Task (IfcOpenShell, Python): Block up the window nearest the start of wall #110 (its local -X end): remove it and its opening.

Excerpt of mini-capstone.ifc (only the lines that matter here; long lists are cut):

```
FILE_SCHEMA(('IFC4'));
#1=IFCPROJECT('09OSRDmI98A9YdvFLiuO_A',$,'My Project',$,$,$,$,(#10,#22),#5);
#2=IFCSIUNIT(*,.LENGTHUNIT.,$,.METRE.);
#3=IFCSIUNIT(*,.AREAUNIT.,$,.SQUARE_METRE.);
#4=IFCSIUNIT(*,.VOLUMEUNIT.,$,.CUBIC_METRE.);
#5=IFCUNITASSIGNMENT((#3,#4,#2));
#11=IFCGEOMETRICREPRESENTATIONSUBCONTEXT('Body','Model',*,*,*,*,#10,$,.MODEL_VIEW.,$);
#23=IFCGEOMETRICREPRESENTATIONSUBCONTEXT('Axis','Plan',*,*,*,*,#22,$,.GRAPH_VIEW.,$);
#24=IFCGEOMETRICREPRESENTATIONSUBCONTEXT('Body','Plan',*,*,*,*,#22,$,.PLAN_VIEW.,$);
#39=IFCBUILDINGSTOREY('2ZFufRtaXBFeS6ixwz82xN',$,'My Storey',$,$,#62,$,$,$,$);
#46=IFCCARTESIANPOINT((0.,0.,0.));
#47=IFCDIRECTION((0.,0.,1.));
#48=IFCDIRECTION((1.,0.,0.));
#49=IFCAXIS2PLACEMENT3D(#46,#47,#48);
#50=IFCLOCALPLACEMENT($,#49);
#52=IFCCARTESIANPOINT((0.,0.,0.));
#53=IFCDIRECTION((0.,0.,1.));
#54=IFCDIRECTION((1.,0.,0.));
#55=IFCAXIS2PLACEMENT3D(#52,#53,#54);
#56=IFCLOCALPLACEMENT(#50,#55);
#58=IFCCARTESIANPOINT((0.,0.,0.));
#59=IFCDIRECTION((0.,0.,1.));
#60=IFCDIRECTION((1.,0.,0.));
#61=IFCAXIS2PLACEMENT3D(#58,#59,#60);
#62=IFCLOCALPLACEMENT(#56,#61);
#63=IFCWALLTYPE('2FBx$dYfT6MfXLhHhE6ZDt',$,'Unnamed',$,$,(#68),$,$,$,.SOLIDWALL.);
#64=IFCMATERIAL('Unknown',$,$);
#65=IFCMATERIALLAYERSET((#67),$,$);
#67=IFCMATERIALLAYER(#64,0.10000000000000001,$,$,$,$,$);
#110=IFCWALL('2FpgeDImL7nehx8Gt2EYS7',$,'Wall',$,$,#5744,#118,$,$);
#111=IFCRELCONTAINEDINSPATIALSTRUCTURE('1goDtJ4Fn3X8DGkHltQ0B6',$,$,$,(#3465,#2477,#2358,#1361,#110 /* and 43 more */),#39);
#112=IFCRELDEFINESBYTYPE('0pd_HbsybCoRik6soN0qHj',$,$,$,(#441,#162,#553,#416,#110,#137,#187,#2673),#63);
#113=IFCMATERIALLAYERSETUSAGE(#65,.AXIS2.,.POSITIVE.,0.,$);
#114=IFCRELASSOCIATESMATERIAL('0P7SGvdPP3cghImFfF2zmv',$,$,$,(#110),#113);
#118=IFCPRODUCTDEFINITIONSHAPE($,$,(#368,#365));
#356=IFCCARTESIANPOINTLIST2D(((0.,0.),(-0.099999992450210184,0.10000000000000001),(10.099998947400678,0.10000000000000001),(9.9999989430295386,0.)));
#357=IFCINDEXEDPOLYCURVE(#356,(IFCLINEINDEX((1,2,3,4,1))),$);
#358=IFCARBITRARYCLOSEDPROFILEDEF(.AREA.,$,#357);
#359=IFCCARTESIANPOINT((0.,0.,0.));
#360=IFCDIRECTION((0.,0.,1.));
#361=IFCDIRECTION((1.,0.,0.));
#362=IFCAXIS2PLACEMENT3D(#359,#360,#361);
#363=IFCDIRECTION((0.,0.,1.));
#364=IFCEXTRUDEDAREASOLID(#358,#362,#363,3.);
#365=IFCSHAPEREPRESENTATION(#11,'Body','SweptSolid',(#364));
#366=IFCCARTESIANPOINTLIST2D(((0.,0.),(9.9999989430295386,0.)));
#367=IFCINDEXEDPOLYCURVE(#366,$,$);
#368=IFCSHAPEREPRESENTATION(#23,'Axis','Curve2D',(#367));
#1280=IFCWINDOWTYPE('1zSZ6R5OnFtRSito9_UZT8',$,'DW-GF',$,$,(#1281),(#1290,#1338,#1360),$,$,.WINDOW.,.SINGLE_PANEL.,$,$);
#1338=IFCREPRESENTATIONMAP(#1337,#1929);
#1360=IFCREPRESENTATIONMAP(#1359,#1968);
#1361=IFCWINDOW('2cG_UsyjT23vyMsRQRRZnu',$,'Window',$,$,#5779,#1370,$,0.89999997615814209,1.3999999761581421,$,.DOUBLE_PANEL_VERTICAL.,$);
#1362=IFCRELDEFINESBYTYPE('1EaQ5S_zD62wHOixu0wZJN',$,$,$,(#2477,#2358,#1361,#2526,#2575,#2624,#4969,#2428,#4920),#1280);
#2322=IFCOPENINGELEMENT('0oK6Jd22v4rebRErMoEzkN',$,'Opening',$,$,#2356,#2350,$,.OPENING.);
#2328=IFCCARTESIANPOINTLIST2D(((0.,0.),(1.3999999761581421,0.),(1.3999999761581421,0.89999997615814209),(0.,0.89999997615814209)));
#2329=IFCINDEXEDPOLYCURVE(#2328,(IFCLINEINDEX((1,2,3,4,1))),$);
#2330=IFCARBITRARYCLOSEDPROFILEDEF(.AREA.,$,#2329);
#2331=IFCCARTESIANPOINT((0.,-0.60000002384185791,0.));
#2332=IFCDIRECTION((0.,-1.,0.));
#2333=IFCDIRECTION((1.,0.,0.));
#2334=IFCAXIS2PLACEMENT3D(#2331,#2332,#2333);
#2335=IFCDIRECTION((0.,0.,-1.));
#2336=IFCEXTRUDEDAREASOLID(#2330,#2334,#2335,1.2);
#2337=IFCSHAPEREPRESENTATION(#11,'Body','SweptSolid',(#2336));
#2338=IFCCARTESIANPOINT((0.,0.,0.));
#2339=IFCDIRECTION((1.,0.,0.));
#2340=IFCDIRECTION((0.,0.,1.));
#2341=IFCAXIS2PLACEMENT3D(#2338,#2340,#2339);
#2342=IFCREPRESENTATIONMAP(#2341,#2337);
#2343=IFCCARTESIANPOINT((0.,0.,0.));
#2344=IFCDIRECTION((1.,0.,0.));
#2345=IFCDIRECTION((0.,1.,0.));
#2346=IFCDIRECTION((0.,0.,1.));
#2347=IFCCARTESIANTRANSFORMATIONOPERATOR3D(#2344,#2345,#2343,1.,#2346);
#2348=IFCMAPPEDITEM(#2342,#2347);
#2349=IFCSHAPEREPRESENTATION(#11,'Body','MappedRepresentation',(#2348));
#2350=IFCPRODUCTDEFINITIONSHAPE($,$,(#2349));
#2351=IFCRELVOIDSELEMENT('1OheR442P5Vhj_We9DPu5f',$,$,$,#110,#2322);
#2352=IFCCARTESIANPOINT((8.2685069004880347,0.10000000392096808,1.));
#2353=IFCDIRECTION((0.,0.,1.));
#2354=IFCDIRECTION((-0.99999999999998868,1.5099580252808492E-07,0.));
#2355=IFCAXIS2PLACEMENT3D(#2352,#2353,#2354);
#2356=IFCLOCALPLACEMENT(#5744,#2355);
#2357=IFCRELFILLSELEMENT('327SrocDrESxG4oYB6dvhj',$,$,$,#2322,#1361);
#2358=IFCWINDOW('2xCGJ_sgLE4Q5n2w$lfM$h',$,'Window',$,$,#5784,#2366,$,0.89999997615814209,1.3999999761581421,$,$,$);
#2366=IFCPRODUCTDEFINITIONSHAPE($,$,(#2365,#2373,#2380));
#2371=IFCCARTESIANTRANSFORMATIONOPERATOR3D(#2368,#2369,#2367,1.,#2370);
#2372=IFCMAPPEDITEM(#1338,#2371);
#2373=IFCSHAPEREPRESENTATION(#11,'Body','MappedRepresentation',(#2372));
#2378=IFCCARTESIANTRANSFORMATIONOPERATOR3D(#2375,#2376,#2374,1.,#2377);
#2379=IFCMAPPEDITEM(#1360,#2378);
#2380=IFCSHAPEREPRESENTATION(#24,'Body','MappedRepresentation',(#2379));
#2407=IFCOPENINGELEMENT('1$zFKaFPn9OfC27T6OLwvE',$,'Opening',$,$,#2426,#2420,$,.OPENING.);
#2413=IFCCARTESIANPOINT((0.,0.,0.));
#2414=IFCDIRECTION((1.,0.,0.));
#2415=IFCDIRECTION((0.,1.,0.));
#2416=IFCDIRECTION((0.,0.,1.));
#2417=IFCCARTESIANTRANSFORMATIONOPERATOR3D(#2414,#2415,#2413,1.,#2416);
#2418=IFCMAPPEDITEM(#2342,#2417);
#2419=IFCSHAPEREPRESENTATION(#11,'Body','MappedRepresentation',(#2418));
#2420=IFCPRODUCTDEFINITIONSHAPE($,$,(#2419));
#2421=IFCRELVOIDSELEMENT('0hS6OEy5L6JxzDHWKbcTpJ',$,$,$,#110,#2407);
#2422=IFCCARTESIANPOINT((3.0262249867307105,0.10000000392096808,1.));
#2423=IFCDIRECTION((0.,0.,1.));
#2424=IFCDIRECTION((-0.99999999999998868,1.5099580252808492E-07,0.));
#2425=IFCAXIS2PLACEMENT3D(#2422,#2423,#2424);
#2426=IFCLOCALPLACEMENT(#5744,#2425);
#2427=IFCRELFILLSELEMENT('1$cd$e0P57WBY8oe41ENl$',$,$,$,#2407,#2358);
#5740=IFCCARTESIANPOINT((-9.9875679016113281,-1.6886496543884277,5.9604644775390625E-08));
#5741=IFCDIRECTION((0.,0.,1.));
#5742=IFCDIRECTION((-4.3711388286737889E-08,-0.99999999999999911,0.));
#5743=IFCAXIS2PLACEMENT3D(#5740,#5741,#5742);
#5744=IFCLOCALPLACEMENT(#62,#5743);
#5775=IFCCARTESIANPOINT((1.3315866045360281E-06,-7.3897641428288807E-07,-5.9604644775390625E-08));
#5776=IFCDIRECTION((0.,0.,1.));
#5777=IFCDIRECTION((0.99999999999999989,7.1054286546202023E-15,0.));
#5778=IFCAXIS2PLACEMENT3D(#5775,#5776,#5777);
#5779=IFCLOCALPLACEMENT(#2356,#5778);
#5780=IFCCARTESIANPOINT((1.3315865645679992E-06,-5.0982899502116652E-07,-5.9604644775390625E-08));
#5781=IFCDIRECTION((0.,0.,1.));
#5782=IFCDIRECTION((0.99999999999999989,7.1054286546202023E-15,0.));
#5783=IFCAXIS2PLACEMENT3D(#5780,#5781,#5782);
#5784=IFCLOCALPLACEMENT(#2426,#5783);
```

```python
import ifcopenshell
import ifcopenshell.api.feature
import ifcopenshell.api.root
import ifcopenshell.geom
import ifcopenshell.util.shape

model = ifcopenshell.open("mini-capstone.ifc")
settings = ifcopenshell.geom.settings()


def volume(element):
    """Net volume in cubic metres, openings subtracted."""
    shape = ifcopenshell.geom.create_shape(settings, element)
    return ifcopenshell.util.shape.get_volume(shape.geometry)


window = model.by_guid("2xCGJ_sgLE4Q5n2w$lfM$h")
opening = window.FillsVoids[0].RelatingOpeningElement
wall = opening.VoidsElements[0].RelatingBuildingElement
before = volume(wall)

ifcopenshell.api.root.remove_product(model, product=window)
ifcopenshell.api.feature.remove_feature(model, feature=opening)

after = volume(wall)

print(f"wall volume {before:.3f} -> {after:.3f} m3")

model.write("mini-capstone_edited.ifc")
```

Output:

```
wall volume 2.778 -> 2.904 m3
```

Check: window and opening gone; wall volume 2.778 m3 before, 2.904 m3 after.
